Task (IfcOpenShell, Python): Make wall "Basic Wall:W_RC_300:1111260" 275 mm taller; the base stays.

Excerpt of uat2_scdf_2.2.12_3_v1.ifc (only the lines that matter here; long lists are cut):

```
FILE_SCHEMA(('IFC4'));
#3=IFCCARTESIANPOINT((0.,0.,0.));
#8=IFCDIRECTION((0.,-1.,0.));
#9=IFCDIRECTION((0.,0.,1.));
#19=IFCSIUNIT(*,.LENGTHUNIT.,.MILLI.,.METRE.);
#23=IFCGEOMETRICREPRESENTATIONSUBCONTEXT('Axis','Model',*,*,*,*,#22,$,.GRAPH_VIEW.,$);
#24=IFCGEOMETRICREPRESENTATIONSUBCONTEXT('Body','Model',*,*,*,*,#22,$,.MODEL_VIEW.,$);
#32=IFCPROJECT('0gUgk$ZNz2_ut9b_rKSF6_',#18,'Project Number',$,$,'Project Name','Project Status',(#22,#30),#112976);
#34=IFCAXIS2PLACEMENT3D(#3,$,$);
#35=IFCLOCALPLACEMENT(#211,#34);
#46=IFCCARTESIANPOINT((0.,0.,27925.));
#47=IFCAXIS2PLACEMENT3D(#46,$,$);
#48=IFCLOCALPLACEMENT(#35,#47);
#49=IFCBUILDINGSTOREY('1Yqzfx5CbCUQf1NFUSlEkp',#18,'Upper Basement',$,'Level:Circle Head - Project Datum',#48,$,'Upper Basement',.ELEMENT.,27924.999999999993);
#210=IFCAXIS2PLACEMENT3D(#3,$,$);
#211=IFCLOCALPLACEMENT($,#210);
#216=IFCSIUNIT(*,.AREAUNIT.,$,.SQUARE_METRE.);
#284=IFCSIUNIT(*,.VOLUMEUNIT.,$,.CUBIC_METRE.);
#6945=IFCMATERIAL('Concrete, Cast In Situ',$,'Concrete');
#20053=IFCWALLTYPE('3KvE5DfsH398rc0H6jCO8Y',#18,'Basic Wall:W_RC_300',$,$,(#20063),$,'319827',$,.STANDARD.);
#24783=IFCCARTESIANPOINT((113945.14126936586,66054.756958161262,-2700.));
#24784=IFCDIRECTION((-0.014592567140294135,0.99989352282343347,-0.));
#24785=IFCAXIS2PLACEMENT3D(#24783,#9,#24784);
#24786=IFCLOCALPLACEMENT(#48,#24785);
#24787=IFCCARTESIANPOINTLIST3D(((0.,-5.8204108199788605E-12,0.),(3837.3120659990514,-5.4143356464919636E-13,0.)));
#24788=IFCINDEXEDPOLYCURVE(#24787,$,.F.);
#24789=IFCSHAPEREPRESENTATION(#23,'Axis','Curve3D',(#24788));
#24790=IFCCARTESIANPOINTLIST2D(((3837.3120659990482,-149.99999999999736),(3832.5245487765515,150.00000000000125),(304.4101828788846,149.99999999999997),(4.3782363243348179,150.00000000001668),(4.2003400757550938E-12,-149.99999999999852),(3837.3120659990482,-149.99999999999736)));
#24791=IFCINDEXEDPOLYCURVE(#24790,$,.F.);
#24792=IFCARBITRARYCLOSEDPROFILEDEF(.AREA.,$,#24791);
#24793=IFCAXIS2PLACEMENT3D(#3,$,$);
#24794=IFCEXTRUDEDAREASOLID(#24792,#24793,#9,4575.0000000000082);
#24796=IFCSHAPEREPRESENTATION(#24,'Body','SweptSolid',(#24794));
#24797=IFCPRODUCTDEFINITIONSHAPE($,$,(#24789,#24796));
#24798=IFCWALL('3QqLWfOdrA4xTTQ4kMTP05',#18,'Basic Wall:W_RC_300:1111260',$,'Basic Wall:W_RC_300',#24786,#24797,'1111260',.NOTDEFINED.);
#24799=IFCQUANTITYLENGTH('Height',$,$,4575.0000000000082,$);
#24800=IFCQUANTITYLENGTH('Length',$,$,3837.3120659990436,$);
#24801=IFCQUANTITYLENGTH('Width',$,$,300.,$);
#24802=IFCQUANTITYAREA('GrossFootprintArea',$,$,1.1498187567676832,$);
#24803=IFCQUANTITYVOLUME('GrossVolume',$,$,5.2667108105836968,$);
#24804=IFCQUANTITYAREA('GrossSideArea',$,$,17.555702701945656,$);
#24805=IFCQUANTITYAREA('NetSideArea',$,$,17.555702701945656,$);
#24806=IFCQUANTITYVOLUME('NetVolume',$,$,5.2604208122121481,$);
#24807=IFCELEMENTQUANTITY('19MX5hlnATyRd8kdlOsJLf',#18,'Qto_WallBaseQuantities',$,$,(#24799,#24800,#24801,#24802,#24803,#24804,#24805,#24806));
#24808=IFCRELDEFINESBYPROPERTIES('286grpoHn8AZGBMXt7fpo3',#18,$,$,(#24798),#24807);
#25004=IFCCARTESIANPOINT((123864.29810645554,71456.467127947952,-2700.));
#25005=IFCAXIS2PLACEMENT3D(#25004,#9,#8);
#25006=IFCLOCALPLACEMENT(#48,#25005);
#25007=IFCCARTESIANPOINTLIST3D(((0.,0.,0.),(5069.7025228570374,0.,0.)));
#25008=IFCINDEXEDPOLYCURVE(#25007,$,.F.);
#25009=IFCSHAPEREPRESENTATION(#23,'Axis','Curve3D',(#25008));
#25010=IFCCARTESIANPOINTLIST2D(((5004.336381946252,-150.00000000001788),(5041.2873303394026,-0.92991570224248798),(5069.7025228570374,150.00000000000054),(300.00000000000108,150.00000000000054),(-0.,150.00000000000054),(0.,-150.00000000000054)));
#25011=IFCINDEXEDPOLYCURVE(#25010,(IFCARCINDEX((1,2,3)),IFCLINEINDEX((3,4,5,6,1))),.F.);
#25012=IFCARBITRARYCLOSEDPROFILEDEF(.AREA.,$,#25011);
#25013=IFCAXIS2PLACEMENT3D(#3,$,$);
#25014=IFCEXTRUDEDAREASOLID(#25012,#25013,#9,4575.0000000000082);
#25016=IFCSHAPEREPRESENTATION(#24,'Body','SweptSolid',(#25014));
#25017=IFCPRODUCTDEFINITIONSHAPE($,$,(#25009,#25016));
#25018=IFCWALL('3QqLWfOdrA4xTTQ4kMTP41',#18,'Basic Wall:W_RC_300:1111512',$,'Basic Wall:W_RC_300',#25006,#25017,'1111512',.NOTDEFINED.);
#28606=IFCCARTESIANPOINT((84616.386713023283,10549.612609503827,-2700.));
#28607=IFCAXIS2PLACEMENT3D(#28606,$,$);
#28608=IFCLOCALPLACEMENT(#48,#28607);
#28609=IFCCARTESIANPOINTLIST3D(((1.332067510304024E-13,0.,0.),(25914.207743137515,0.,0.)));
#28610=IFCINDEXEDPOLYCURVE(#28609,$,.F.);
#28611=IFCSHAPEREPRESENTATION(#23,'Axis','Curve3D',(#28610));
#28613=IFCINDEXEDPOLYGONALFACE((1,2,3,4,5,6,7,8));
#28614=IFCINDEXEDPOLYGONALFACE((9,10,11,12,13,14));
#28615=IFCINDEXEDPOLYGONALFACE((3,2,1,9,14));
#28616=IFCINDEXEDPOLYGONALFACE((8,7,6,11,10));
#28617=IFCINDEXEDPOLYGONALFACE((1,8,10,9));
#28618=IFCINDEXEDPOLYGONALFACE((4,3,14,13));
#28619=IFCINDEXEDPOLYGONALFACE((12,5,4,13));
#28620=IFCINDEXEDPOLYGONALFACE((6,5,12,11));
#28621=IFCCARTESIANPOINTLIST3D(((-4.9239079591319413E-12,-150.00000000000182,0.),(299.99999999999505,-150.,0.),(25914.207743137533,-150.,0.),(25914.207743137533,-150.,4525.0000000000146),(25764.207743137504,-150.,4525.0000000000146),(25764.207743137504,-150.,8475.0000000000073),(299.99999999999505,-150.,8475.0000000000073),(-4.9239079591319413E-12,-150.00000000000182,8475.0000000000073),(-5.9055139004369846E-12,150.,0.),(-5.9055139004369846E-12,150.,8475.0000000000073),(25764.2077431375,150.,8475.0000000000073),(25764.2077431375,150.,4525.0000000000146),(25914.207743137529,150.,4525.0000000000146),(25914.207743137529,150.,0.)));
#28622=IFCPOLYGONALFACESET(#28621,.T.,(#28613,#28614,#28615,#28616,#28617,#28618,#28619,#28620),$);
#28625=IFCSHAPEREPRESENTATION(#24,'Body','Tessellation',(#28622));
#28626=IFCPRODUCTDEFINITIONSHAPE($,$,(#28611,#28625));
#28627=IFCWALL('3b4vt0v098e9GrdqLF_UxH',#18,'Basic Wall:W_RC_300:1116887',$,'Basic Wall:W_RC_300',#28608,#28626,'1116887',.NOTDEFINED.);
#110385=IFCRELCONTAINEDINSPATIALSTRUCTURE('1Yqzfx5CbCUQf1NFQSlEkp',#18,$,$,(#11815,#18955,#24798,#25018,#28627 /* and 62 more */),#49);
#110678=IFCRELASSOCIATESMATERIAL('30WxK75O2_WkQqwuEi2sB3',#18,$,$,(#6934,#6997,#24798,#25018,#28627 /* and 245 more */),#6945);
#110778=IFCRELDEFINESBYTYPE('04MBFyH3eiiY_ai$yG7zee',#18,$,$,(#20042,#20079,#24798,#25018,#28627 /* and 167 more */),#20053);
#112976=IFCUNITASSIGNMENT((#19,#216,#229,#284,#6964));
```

```python
import ifcopenshell
import ifcopenshell.api.pset
import ifcopenshell.geom
import ifcopenshell.util.element
import ifcopenshell.util.representation
import ifcopenshell.util.shape
import ifcopenshell.util.unit

model = ifcopenshell.open("uat2_scdf_2.2.12_3_v1.ifc")
unit_scale = ifcopenshell.util.unit.calculate_unit_scale(model)
area_scale = ifcopenshell.util.unit.calculate_unit_scale(model, "AREAUNIT")
volume_scale = ifcopenshell.util.unit.calculate_unit_scale(model, "VOLUMEUNIT")
settings = ifcopenshell.geom.settings()


def volume(element):
    """Net volume in cubic metres, openings subtracted."""
    shape = ifcopenshell.geom.create_shape(settings, element)
    return ifcopenshell.util.shape.get_volume(shape.geometry)


wall = model.by_guid("3QqLWfOdrA4xTTQ4kMTP05")
before = volume(wall)

body = ifcopenshell.util.representation.get_representation(wall, "Model", "Body")
solid = body.Items[0]
old_height = solid.Depth
solid.Depth += 275.0
after = volume(wall)
thickness = 0.3  # wall thickness in metres

# Update the stored height, areas and volumes.
qto = model.by_id(ifcopenshell.util.element.get_pset(wall, "Qto_WallBaseQuantities", should_inherit=False)["id"])
ifcopenshell.api.pset.edit_qto(model, qto=qto, properties={
    "Height": solid.Depth,
    "GrossVolume": ifcopenshell.util.element.get_pset(wall, "Qto_WallBaseQuantities", "GrossVolume") * solid.Depth / old_height,
    "GrossSideArea": ifcopenshell.util.element.get_pset(wall, "Qto_WallBaseQuantities", "GrossSideArea") * solid.Depth / old_height,
    "NetSideArea": after / thickness / area_scale,
    "NetVolume": after / volume_scale,
})

print(f"height {old_height:g} -> {solid.Depth:g}, volume {before:.3f} -> {after:.3f} m3")

model.write("uat2_scdf_2.2.12_3_v1-out.ifc")
```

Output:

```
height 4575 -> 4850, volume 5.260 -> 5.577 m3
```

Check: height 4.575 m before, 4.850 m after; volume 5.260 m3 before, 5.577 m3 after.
